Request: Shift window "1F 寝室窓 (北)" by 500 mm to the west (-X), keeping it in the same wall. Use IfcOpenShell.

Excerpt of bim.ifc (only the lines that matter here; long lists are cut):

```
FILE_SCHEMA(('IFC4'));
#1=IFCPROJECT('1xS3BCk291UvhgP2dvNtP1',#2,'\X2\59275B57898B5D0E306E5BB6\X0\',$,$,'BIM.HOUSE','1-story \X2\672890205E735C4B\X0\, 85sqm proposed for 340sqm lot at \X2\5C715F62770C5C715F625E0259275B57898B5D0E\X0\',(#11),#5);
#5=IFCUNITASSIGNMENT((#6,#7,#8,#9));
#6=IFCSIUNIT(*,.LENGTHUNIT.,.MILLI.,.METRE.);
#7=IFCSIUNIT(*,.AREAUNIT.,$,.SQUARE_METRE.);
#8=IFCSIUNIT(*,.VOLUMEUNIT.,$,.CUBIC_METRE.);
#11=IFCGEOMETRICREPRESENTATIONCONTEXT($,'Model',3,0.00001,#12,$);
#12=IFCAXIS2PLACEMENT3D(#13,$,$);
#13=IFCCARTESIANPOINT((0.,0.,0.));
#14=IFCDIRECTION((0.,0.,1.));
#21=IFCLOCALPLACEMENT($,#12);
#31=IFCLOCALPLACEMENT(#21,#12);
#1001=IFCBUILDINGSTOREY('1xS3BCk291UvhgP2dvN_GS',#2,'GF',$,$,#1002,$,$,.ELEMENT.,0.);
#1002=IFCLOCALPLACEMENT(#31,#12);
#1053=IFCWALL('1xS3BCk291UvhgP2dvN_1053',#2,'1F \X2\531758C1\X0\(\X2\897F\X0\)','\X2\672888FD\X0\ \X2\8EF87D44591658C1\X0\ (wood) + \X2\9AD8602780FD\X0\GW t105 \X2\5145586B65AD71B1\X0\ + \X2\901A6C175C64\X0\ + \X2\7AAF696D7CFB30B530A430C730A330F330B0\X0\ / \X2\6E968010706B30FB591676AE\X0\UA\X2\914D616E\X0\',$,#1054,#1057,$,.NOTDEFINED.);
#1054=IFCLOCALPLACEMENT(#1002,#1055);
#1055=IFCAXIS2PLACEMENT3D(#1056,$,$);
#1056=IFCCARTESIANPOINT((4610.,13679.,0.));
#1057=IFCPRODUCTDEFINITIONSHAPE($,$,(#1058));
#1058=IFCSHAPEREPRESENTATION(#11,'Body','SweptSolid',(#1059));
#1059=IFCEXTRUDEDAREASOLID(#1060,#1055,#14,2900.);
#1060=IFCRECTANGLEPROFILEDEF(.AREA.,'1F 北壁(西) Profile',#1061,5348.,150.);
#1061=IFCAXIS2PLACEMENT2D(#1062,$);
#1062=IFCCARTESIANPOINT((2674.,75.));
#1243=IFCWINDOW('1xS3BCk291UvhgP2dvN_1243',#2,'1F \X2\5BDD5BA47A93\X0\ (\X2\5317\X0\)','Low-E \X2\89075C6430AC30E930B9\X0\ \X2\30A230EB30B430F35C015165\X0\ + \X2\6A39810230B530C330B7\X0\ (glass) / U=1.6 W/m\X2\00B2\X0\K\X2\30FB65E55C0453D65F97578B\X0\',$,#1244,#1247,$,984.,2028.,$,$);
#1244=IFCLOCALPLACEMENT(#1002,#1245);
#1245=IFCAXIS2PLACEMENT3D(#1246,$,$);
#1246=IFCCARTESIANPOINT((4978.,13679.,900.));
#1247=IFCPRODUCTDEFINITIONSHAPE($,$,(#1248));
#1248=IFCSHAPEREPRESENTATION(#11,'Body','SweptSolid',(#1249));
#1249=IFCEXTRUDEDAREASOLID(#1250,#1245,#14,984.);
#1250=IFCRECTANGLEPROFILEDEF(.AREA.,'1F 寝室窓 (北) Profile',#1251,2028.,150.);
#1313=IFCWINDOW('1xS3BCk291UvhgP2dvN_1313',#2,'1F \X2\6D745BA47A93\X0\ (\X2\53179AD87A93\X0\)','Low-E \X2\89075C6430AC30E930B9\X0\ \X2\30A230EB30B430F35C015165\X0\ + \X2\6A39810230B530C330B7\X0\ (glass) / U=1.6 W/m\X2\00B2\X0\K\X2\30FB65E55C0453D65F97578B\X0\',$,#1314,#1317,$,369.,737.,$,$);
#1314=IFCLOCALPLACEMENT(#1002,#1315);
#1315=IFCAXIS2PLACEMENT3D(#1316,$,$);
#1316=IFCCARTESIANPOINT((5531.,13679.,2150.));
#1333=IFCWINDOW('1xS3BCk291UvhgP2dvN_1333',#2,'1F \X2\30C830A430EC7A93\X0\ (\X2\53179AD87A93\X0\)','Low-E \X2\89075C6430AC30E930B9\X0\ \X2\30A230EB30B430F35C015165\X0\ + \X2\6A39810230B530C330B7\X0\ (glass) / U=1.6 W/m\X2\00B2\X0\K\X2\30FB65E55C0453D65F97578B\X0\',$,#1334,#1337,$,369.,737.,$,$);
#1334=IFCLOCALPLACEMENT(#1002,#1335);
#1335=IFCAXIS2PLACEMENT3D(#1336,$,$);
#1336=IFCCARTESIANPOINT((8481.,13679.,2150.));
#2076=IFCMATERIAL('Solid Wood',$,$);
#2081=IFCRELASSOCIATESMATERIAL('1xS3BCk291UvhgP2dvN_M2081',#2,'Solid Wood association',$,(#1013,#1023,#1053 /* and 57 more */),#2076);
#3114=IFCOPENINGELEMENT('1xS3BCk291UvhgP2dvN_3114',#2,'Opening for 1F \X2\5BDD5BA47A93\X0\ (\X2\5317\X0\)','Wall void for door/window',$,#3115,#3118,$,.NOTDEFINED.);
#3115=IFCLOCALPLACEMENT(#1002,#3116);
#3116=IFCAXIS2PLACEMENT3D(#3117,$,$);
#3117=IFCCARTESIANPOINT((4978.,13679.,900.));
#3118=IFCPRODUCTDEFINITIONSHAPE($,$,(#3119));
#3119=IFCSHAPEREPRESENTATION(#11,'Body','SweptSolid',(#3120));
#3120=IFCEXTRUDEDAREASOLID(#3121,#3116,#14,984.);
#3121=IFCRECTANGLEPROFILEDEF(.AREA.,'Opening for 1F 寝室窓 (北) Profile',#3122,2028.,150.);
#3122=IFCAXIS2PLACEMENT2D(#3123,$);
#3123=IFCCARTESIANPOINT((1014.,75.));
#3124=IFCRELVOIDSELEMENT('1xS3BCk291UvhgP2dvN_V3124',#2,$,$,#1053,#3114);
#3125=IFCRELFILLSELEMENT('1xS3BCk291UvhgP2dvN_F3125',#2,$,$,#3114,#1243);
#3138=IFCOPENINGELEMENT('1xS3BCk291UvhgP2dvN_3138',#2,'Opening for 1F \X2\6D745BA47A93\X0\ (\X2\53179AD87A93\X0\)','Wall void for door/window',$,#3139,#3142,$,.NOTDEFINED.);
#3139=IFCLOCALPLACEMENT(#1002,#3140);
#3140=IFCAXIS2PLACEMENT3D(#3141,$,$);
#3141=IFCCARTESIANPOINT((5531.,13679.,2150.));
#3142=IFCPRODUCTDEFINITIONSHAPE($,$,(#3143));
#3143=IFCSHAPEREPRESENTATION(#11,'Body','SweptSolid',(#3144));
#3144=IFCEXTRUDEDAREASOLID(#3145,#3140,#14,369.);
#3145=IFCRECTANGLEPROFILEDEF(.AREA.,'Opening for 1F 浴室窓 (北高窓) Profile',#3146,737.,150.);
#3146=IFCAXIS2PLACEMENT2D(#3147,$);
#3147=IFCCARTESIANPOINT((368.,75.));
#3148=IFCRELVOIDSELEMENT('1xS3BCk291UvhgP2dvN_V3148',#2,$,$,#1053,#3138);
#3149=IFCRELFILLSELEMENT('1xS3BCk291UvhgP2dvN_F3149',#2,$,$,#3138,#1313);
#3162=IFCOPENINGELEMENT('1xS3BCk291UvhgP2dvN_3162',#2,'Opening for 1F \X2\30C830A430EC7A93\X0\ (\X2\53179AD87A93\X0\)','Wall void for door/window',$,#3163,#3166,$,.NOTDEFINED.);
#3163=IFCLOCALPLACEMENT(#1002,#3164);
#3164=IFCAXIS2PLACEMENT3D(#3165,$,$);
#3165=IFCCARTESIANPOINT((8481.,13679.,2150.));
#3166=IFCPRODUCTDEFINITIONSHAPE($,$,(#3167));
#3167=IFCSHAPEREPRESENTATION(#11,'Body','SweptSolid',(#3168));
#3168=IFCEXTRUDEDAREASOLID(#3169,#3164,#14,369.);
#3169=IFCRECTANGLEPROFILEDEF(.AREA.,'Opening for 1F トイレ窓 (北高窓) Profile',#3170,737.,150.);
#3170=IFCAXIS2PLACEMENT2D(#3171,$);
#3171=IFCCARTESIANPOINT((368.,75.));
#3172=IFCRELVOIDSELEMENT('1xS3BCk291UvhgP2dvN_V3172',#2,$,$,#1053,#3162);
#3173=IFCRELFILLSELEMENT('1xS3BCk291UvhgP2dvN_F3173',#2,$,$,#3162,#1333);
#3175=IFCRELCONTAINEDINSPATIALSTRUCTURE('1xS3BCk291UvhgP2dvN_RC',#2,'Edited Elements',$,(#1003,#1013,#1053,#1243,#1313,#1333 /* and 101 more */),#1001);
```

```python
import ifcopenshell
import ifcopenshell.api.geometry
import ifcopenshell.util.placement
import ifcopenshell.util.unit

model = ifcopenshell.open("bim.ifc")
unit_scale = ifcopenshell.util.unit.calculate_unit_scale(model)

window = model.by_id(1243)
opening = window.FillsVoids[0].RelatingOpeningElement
wall = opening.VoidsElements[0].RelatingBuildingElement

wall_matrix = ifcopenshell.util.placement.get_local_placement(wall.ObjectPlacement)
shift = wall_matrix[:3, 0] * -0.5 / unit_scale
before = ifcopenshell.util.placement.get_local_placement(window.ObjectPlacement)[:3, 3].copy()

# The window is not placed relative to its opening, so move both.
for product in (opening, window):
    matrix = ifcopenshell.util.placement.get_local_placement(product.ObjectPlacement)
    matrix[:3, 3] += shift
    ifcopenshell.api.geometry.edit_object_placement(model, product=product, matrix=matrix, is_si=False)

after = ifcopenshell.util.placement.get_local_placement(window.ObjectPlacement)[:3, 3]
print("window moved by", (after - before).round(3) + 0.0)

model.write("bim-out.ifc")
```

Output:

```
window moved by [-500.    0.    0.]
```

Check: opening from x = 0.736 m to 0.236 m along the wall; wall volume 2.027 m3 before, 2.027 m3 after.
